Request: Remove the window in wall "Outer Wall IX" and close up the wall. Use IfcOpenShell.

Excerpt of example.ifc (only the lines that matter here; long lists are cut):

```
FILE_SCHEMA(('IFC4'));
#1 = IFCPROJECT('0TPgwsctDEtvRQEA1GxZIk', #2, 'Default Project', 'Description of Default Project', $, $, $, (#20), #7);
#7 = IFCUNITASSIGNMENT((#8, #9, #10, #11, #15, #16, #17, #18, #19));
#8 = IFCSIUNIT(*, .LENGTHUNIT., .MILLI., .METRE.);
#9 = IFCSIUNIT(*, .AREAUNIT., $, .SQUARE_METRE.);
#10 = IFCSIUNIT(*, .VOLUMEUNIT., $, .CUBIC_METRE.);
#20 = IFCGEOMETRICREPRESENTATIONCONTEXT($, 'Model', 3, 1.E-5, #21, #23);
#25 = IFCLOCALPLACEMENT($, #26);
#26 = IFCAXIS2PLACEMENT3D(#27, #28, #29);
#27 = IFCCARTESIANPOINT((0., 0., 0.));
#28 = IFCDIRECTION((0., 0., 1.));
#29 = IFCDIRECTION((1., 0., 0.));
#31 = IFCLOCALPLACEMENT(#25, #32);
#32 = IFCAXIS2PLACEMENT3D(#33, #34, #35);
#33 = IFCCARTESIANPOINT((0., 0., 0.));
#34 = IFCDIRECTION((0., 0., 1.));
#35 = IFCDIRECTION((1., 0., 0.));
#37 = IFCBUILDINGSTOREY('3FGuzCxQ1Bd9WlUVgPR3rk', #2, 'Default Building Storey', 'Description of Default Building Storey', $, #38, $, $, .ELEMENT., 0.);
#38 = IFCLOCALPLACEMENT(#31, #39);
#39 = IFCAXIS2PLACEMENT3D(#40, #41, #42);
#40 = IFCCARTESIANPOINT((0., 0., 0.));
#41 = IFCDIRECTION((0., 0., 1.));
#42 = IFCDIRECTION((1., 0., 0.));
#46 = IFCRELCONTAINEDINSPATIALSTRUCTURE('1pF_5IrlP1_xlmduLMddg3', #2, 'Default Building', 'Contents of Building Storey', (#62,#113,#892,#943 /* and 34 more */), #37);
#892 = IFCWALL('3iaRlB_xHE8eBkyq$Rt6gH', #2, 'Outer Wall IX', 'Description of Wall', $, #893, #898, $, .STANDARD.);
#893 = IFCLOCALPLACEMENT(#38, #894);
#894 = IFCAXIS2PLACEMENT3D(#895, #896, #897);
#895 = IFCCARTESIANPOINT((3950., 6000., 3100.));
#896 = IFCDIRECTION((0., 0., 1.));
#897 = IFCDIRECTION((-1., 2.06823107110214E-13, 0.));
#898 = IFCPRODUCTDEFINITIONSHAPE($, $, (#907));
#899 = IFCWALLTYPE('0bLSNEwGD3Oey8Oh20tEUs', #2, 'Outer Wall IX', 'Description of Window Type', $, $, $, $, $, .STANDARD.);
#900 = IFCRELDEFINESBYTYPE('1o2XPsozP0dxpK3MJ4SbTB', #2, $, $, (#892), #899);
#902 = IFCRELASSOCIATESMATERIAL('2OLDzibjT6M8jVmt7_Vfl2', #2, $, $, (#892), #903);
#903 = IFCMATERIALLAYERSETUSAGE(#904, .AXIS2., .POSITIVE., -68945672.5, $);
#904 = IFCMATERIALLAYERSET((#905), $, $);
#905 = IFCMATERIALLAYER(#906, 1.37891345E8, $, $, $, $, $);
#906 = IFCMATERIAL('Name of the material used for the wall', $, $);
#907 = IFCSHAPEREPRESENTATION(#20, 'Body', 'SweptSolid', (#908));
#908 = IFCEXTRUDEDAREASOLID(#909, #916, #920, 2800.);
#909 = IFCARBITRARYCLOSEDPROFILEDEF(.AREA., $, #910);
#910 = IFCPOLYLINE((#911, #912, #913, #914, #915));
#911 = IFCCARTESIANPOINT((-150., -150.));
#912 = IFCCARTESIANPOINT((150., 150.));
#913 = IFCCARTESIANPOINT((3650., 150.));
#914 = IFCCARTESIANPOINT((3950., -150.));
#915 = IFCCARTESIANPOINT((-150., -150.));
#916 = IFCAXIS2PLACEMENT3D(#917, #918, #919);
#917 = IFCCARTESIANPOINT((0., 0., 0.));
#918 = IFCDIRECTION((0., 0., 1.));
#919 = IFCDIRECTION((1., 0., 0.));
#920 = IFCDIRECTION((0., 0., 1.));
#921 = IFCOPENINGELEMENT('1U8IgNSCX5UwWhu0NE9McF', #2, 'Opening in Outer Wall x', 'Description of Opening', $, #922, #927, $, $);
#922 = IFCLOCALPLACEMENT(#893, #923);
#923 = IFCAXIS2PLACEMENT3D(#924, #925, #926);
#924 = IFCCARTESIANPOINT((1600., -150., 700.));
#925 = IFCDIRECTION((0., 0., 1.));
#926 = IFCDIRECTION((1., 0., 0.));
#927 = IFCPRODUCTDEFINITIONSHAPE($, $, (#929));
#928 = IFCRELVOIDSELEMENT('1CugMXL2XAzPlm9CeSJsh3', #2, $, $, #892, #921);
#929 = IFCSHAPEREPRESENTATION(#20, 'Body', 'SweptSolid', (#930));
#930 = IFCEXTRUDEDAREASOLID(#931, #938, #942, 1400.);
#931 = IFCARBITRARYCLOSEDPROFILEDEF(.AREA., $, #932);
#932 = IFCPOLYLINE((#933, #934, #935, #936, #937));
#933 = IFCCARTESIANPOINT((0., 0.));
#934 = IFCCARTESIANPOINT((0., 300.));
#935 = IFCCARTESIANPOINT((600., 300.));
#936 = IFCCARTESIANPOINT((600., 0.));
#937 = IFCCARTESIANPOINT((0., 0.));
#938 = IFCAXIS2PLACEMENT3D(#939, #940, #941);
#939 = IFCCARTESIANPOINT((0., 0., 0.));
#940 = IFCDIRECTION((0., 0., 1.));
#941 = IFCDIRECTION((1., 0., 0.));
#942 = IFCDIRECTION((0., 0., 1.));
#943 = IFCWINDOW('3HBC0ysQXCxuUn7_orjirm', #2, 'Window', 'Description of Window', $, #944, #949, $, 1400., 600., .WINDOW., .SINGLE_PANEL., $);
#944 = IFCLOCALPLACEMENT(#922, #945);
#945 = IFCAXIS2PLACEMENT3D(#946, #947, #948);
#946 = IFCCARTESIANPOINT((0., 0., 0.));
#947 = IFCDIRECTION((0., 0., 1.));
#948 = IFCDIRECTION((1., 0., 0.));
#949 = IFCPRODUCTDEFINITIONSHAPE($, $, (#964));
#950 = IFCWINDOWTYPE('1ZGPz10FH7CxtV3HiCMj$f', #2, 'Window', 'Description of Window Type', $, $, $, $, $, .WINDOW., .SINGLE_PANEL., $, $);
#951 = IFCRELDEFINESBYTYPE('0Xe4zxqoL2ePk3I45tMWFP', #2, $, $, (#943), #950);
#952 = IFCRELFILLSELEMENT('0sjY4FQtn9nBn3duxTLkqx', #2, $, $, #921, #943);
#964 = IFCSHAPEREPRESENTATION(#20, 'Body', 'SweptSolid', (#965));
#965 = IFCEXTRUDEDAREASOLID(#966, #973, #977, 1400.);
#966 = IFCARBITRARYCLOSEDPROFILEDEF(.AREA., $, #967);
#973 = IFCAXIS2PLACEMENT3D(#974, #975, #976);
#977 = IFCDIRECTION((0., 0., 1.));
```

```python
import ifcopenshell
import ifcopenshell.api.feature
import ifcopenshell.api.root
import ifcopenshell.geom
import ifcopenshell.util.shape

model = ifcopenshell.open("example.ifc")
settings = ifcopenshell.geom.settings()


def volume(element):
    """Net volume in cubic metres, openings subtracted."""
    shape = ifcopenshell.geom.create_shape(settings, element)
    return ifcopenshell.util.shape.get_volume(shape.geometry)


window = model.by_guid("3HBC0ysQXCxuUn7_orjirm")
opening = window.FillsVoids[0].RelatingOpeningElement
wall = opening.VoidsElements[0].RelatingBuildingElement
before = volume(wall)

ifcopenshell.api.root.remove_product(model, product=window)
ifcopenshell.api.feature.remove_feature(model, feature=opening)

after = volume(wall)

print(f"wall volume {before:.3f} -> {after:.3f} m3")

model.write("example_rev.ifc")
```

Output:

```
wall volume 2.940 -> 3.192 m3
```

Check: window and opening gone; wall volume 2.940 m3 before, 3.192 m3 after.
